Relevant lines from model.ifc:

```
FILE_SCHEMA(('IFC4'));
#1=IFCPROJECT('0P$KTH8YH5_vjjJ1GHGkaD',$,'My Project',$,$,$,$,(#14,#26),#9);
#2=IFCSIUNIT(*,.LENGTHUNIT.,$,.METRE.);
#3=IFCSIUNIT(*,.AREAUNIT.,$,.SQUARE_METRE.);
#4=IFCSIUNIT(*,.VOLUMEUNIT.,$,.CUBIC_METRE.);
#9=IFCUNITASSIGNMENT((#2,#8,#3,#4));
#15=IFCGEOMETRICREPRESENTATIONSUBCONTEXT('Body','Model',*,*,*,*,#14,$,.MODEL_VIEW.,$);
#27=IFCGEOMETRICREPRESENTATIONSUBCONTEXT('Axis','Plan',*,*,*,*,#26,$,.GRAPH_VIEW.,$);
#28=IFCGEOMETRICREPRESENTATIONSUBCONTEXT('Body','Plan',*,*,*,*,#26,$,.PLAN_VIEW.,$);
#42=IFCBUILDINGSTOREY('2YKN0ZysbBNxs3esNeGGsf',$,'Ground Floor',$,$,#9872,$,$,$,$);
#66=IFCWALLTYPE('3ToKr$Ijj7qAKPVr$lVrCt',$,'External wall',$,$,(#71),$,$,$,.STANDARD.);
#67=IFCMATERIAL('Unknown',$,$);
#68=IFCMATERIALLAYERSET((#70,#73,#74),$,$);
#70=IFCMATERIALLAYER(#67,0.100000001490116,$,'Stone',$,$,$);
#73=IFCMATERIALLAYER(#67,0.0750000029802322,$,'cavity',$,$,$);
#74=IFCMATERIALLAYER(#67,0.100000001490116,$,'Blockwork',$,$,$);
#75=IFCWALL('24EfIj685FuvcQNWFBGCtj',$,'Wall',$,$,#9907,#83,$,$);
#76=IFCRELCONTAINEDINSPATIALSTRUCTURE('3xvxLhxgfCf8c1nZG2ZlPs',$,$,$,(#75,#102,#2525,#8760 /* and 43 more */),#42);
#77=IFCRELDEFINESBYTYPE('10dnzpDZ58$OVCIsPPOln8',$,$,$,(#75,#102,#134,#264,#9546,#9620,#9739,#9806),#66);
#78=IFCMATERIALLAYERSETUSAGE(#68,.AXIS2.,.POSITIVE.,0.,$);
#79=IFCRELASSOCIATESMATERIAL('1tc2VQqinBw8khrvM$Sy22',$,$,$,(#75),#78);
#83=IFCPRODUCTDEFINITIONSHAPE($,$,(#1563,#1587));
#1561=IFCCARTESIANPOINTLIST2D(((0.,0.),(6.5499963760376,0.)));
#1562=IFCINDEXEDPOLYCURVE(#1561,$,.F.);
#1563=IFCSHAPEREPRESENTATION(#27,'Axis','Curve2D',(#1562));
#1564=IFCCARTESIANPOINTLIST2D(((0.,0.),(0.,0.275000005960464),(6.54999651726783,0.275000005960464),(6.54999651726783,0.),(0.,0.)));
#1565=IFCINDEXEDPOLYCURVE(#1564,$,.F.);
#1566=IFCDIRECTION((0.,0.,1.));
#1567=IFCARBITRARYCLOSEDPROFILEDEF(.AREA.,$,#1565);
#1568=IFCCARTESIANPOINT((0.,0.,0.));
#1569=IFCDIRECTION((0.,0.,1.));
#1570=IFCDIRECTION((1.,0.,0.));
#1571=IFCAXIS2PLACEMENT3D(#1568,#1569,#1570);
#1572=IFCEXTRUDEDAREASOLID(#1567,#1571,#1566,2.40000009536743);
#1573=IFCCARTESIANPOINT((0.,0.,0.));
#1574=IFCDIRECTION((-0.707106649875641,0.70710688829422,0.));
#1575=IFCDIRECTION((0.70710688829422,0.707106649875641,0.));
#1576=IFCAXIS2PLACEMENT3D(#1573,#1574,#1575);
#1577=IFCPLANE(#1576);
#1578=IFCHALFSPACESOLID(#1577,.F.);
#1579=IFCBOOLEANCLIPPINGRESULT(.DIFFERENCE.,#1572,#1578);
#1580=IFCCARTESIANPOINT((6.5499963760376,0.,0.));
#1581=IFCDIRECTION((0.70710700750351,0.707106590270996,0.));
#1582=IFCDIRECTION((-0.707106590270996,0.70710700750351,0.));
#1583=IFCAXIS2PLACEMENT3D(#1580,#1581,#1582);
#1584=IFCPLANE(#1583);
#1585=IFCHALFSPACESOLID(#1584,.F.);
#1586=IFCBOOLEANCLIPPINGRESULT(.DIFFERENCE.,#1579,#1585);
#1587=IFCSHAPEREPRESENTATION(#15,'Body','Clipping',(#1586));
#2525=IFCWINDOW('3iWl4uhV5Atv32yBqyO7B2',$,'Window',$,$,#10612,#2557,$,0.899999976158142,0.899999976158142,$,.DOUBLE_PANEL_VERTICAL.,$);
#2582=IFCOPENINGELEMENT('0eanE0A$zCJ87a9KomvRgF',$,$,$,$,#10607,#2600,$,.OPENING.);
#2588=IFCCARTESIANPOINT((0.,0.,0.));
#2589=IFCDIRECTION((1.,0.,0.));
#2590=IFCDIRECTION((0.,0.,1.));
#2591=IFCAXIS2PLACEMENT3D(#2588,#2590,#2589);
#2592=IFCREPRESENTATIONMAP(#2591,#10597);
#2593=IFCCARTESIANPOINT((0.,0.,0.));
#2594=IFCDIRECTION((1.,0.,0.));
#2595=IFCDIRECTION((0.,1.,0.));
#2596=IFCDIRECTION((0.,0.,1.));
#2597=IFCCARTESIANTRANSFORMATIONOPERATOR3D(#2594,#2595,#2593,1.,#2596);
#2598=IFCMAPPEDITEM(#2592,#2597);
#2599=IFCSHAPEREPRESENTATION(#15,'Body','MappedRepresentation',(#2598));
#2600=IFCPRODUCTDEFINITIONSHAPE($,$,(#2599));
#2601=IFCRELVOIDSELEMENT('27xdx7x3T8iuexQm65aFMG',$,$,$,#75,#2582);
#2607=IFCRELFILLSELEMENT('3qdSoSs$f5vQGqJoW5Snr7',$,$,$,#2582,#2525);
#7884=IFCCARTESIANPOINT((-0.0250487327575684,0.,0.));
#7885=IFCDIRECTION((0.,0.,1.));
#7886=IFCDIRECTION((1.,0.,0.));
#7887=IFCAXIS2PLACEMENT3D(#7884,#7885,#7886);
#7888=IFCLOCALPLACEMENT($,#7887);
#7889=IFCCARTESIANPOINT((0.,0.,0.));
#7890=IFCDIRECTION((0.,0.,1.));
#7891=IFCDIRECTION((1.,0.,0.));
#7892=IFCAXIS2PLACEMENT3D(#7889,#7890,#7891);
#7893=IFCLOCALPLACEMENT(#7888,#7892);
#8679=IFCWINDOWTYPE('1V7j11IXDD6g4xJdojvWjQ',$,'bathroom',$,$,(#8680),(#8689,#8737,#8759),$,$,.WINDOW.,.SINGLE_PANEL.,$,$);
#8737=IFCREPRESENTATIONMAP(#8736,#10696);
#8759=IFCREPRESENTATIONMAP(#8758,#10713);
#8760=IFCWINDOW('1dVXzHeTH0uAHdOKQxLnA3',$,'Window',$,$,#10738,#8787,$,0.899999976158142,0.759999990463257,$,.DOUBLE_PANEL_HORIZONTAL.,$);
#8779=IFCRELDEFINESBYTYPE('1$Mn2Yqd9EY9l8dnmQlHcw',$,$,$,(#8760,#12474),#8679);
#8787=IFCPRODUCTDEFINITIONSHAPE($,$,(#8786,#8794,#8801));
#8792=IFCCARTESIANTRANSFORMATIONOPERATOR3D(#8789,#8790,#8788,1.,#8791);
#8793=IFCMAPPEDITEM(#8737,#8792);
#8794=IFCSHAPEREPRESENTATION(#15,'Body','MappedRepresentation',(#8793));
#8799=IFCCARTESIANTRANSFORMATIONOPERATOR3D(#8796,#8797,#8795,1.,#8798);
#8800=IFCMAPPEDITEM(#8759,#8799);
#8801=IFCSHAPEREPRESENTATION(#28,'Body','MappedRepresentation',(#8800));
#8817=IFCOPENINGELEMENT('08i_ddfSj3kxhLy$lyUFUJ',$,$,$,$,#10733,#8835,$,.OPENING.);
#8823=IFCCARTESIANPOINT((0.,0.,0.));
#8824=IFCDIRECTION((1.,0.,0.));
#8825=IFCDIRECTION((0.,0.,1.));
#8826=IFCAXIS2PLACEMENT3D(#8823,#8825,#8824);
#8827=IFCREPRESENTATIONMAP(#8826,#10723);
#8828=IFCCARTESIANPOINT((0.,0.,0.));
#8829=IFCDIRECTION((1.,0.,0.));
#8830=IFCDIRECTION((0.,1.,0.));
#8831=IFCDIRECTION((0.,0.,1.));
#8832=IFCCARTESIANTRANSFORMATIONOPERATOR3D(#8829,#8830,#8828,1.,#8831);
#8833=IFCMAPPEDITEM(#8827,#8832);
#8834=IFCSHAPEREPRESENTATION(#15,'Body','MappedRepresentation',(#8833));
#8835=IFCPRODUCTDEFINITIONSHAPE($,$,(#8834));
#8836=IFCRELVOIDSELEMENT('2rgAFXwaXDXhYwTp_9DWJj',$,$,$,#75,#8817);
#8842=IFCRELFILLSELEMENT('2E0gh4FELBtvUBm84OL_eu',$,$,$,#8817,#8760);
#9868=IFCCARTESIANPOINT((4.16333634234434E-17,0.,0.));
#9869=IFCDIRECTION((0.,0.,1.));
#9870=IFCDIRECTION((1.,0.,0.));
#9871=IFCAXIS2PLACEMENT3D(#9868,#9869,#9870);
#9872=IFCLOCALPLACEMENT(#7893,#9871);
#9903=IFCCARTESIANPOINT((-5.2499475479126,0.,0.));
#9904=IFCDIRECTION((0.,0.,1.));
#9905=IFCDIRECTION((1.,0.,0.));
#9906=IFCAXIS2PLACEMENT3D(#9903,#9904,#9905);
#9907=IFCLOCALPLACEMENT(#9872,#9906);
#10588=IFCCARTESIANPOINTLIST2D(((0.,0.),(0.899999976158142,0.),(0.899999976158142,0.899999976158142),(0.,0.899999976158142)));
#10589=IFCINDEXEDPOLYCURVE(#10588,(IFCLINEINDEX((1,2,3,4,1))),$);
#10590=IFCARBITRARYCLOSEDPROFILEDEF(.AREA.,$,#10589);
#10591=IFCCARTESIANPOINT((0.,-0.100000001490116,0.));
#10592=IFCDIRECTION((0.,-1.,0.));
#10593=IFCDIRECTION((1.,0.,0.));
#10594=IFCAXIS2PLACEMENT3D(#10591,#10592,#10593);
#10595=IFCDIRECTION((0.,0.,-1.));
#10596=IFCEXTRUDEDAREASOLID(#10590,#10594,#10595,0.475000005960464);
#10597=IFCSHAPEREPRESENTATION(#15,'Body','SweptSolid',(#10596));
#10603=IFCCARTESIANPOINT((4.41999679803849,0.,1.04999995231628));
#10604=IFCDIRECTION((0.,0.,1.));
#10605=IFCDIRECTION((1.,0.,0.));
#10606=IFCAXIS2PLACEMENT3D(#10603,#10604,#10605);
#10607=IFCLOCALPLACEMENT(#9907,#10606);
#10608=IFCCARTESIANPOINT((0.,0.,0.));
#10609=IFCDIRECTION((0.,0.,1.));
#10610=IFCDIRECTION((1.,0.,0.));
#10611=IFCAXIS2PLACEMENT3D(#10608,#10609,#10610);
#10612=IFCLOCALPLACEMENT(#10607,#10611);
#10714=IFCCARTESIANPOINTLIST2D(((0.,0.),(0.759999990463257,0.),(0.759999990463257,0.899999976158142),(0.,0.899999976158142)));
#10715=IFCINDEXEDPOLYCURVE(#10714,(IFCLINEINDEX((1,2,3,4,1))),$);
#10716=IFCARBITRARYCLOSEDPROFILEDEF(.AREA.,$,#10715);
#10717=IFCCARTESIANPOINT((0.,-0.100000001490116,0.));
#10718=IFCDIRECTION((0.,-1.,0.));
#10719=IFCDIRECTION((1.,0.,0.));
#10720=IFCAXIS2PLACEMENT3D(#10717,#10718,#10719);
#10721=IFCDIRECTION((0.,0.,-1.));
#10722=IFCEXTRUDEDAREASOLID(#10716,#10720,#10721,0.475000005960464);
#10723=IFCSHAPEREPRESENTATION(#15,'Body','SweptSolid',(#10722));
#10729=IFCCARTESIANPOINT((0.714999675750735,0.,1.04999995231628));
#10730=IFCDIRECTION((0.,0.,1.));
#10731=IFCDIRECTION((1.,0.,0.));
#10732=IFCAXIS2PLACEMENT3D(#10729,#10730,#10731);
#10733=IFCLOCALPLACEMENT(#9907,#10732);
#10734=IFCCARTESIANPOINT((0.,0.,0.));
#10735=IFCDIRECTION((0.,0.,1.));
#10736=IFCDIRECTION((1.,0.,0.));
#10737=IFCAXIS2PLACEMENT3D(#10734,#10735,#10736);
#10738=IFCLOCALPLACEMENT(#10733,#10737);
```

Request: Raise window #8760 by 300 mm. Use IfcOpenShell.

```python
import numpy as np
import ifcopenshell
import ifcopenshell.api.geometry
import ifcopenshell.util.placement
import ifcopenshell.util.unit

model = ifcopenshell.open("model.ifc")
unit_scale = ifcopenshell.util.unit.calculate_unit_scale(model)

window = model.by_guid("1dVXzHeTH0uAHdOKQxLnA3")
opening = window.FillsVoids[0].RelatingOpeningElement
dz = 0.3 / unit_scale

shift = np.array([0.0, 0.0, dz])
# The window is placed relative to its opening, so it follows when the opening moves.
matrix = ifcopenshell.util.placement.get_local_placement(opening.ObjectPlacement)
matrix[:3, 3] += shift
ifcopenshell.api.geometry.edit_object_placement(
    model, product=opening, matrix=matrix, is_si=False, should_transform_children=True
)

print(f"moved by {dz * unit_scale:+.3f} m")

model.write("model-out.ifc")
```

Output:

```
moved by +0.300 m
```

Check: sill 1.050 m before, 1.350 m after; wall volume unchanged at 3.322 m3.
